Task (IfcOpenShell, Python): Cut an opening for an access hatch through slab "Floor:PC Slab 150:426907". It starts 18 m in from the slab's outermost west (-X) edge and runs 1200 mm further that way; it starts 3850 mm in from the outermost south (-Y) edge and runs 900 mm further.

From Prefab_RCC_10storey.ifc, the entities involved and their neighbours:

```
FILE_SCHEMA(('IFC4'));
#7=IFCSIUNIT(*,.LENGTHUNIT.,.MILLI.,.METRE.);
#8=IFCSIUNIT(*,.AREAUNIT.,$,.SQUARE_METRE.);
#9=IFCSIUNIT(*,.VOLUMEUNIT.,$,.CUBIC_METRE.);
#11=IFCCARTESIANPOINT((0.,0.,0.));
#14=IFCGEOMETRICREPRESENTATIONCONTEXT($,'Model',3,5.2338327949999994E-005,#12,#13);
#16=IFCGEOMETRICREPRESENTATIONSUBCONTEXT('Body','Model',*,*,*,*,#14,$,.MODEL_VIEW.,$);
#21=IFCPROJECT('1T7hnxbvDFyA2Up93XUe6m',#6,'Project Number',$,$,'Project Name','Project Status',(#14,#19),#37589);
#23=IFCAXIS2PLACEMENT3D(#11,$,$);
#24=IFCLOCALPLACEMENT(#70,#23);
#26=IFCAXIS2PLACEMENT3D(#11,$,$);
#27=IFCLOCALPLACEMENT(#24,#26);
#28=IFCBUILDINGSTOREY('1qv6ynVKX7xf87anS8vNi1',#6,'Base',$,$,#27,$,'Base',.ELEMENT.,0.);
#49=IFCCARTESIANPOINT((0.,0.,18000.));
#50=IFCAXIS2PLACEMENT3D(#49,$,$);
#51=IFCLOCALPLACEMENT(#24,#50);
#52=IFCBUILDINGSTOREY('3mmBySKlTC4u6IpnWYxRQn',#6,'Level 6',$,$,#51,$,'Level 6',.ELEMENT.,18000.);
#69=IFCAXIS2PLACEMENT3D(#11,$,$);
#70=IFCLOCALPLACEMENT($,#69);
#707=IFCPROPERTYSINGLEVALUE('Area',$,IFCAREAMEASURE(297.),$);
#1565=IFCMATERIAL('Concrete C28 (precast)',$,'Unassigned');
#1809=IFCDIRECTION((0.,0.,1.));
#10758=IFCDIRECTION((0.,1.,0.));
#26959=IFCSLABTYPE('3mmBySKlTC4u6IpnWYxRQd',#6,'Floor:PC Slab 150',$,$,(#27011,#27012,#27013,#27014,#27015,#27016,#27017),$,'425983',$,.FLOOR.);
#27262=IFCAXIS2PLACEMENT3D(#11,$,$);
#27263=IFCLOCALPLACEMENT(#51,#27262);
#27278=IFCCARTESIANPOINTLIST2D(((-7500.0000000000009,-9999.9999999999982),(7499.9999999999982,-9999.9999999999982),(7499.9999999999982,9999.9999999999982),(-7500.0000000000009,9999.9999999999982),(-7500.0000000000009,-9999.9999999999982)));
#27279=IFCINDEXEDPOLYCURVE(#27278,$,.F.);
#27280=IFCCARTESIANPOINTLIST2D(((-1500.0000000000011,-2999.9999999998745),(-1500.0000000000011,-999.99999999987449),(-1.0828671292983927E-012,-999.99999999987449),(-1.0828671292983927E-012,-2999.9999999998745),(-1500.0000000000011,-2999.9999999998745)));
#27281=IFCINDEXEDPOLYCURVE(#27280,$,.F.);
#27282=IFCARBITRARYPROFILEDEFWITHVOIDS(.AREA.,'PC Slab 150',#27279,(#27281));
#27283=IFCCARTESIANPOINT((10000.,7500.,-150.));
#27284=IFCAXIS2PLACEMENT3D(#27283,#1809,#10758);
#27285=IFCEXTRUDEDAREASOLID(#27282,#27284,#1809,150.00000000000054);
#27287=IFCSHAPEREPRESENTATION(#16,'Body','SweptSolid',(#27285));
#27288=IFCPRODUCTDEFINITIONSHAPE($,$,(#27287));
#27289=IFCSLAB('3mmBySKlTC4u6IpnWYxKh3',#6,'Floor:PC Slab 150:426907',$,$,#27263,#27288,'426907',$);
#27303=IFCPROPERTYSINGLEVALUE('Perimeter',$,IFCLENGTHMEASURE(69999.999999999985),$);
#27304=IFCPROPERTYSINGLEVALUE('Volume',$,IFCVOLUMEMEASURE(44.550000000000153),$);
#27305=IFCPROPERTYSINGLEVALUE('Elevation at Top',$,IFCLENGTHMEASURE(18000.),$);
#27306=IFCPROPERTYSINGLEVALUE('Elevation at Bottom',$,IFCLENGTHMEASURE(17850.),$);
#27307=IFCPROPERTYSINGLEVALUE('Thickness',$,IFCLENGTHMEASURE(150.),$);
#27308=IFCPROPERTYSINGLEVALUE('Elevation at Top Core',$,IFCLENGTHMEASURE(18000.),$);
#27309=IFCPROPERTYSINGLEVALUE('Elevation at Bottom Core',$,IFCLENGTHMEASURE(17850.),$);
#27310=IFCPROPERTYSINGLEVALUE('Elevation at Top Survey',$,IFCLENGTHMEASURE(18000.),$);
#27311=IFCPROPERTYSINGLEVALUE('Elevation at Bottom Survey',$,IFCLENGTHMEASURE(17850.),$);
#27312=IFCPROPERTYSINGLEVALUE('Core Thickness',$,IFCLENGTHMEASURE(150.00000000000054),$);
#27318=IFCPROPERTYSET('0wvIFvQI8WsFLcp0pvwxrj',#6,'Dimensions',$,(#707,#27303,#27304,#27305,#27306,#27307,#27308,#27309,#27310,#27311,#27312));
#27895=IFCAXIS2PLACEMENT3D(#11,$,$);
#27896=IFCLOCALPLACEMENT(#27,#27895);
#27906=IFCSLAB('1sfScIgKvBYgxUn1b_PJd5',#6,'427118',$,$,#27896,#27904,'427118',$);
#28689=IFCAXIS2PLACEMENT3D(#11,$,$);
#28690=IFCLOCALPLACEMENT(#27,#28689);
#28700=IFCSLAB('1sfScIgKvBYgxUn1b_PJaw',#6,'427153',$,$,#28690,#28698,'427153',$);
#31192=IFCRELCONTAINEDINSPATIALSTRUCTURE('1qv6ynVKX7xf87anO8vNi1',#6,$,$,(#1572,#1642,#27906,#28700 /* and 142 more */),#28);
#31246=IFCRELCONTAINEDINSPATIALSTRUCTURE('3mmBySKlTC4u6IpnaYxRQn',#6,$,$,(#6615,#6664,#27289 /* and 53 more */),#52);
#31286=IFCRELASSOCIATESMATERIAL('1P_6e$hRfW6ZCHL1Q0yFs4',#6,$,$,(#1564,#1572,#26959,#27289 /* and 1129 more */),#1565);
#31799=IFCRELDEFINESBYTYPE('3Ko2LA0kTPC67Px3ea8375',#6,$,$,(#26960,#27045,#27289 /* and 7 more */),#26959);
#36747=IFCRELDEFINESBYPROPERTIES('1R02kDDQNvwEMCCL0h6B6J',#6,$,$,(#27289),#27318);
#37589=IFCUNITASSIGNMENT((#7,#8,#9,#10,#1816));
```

```python
import numpy as np
import ifcopenshell
import ifcopenshell.api.feature
import ifcopenshell.api.geometry
import ifcopenshell.api.pset
import ifcopenshell.api.root
import ifcopenshell.geom
import ifcopenshell.util.element
import ifcopenshell.util.placement
import ifcopenshell.util.representation
import ifcopenshell.util.shape
import ifcopenshell.util.unit

model = ifcopenshell.open("Prefab_RCC_10storey.ifc")
unit_scale = ifcopenshell.util.unit.calculate_unit_scale(model)
area_scale = ifcopenshell.util.unit.calculate_unit_scale(model, "AREAUNIT")
volume_scale = ifcopenshell.util.unit.calculate_unit_scale(model, "VOLUMEUNIT")
settings = ifcopenshell.geom.settings()


def volume(element):
    """Net volume in cubic metres, openings subtracted."""
    shape = ifcopenshell.geom.create_shape(settings, element)
    return ifcopenshell.util.shape.get_volume(shape.geometry)


slab = model.by_guid("3mmBySKlTC4u6IpnWYxKh3")
before = volume(slab)

# Extent in the slab's own axes, in metres. The edges named are its -X and -Y sides.
slab_shape = ifcopenshell.geom.create_shape(settings, slab)
vertices = ifcopenshell.util.shape.get_vertices(slab_shape.geometry)
x_min, y_min, bottom = vertices.min(axis=0)
top = vertices[:, 2].max()

opening = ifcopenshell.api.root.create_entity(model, ifc_class="IfcOpeningElement", name="Access hatch opening", predefined_type="OPENING")
context = ifcopenshell.util.representation.get_context(model, "Model", "Body", "MODEL_VIEW")
width, depth = 1.2, 0.9
outline = [(0.0, 0.0), (width, 0.0), (width, depth), (0.0, depth), (0.0, 0.0)]
# Overshoot both faces by 50 mm so the cut is clean.
shape = ifcopenshell.api.geometry.add_slab_representation(
    model, context=context, depth=top - bottom + 0.1, polyline=outline
)
ifcopenshell.api.geometry.assign_representation(model, product=opening, representation=shape)

matrix = ifcopenshell.util.placement.get_local_placement(slab.ObjectPlacement)
matrix[:, 3] = matrix @ np.append(np.array([x_min + 18, y_min + 3.85, bottom - 0.05]) / unit_scale, 1.0)
ifcopenshell.api.geometry.edit_object_placement(model, product=opening, matrix=matrix, is_si=False)
ifcopenshell.api.feature.add_feature(model, feature=opening, element=slab)

after = volume(slab)

# Update the slab's stored quantities.
pset = model.by_id(ifcopenshell.util.element.get_pset(slab, "Dimensions", should_inherit=False)["id"])
ifcopenshell.api.pset.edit_pset(model, pset=pset, properties={
    "Area": model.create_entity("IfcAreaMeasure", after / (top - bottom) / area_scale),
    "Volume": model.create_entity("IfcVolumeMeasure", after / volume_scale),
})

print(f"slab volume {before:.3f} -> {after:.3f} m3")

model.write("Prefab_RCC_10storey_rev.ifc")
```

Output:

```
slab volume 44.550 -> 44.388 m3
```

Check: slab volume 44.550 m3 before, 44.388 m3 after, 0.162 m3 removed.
